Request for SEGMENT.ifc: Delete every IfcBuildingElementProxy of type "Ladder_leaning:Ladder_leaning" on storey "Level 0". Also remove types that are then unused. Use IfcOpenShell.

First a look at what the model holds.

```python
import ifcopenshell
import ifcopenshell.util.element

model = ifcopenshell.open("SEGMENT.ifc")
print(model.schema)
storey = next(s for s in model.by_type("IfcBuildingStorey") if s.Name == "Level 0")
proxies = [e for e in ifcopenshell.util.element.get_decomposition(storey) if e.is_a("IfcBuildingElementProxy")]
seen = {}
for e in proxies:
    element_type = ifcopenshell.util.element.get_type(e)
    name = element_type.Name if element_type not in (None, e) else None
    seen[name] = seen.get(name, 0) + 1
for name, count in sorted(seen.items(), key=str):
    print(count, "x", name)
```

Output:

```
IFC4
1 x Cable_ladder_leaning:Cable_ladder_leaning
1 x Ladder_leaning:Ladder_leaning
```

```python
import ifcopenshell
import ifcopenshell.api.root
import ifcopenshell.util.element

model = ifcopenshell.open("SEGMENT.ifc")

storey = next(s for s in model.by_type("IfcBuildingStorey") if s.Name == "Level 0")
proxies = [e for e in ifcopenshell.util.element.get_decomposition(storey) if e.is_a("IfcBuildingElementProxy")]
targets = [e for e in proxies if (t := ifcopenshell.util.element.get_type(e)) not in (None, e) and t.Name == "Ladder_leaning:Ladder_leaning"]
types = {ifcopenshell.util.element.get_type(e) for e in targets} - {None, *targets}

for e in targets:
    ifcopenshell.api.root.remove_product(model, product=e)
print(len(targets), "removed")

unused = [t for t in types if not ifcopenshell.util.element.get_types(t)]
for t in unused:
    ifcopenshell.api.root.remove_product(model, product=t)
print(len(unused), "unused types removed")

model.write("SEGMENT-out.ifc")
```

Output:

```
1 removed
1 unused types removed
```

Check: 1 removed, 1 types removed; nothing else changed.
